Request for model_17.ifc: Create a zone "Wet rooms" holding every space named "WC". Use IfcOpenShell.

First a look at what the model holds.

```python
import ifcopenshell

model = ifcopenshell.open("model_17.ifc")
print(model.schema)
seen = {}
for space in model.by_type("IfcSpace"):
    seen[space.LongName] = seen.get(space.LongName, 0) + 1
for name, count in sorted(seen.items(), key=str):
    print(count, "x", name)
print("zones:", [z.Name for z in model.by_type("IfcZone")][:20])
```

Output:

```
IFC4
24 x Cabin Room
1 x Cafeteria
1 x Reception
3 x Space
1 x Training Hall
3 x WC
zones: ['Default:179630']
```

```python
import ifcopenshell
import ifcopenshell.api.group
import ifcopenshell.api.root

model = ifcopenshell.open("model_17.ifc")

names = {"WC"}
spaces = [s for s in model.by_type("IfcSpace") if s.LongName in names]

zone = ifcopenshell.api.root.create_entity(model, ifc_class="IfcZone", name="Wet rooms")
ifcopenshell.api.group.assign_group(model, products=spaces, group=zone)
print(len(spaces), "spaces in", zone.Name)

model.write("model_17_updated.ifc")
```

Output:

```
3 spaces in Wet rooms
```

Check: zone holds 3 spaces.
